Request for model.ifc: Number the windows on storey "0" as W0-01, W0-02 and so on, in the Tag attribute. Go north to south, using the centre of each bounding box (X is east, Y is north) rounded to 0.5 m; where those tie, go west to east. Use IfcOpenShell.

First a look at what the model holds.

```python
import ifcopenshell
import ifcopenshell.util.element
import ifcopenshell.util.placement

model = ifcopenshell.open("model.ifc")
print(model.schema)
storey = next(s for s in model.by_type("IfcBuildingStorey") if s.Name == "0")
windows = [e for e in ifcopenshell.util.element.get_decomposition(storey) if e.is_a("IfcWindow")]
for e in sorted(windows, key=lambda e: e.id()):
    origin = ifcopenshell.util.placement.get_local_placement(e.ObjectPlacement)[:3, 3]
    print(e.id(), e.Tag, e.Name, origin.round(2) + 0.0, sep=" | ")
```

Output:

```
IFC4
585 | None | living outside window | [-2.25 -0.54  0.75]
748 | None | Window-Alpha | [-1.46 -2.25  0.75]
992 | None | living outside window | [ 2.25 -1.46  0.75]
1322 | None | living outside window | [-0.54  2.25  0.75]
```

```python
import ifcopenshell
import ifcopenshell.geom
import ifcopenshell.util.element
import ifcopenshell.util.shape

model = ifcopenshell.open("model.ifc")
settings = ifcopenshell.geom.settings()
settings.set("use-world-coords", True)


def centre(element):
    shape = ifcopenshell.geom.create_shape(settings, element)
    return ifcopenshell.util.shape.get_bbox_centroid(shape.geometry)


storey = next(s for s in model.by_type("IfcBuildingStorey") if s.Name == "0")
windows = [e for e in ifcopenshell.util.element.get_decomposition(storey) if e.is_a("IfcWindow")]

# Insertion points can sit at a corner or the storey origin, so sort by the geometry (in metres).
centres = {e: centre(e) for e in windows}
windows.sort(key=lambda e: (-round(centres[e][1] / 0.5), centres[e][0]))

for i, e in enumerate(windows, start=1):
    number = f"W0-{i:02d}"
    e.Tag = number
    print(e.id(), number)

model.write("model_rev.ifc")
```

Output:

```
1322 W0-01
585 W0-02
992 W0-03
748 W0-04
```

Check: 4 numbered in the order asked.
